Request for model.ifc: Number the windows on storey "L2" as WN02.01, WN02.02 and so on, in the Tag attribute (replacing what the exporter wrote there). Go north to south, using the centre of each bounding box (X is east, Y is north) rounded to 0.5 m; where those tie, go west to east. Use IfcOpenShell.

First a look at what the model holds.

```python
import ifcopenshell
import ifcopenshell.util.element
import ifcopenshell.util.placement

model = ifcopenshell.open("model.ifc")
print(model.schema)
storey = next(s for s in model.by_type("IfcBuildingStorey") if s.Name == "L2")
windows = [e for e in ifcopenshell.util.element.get_decomposition(storey) if e.is_a("IfcWindow")]
for e in sorted(windows, key=lambda e: e.id()):
    origin = ifcopenshell.util.placement.get_local_placement(e.ObjectPlacement)[:3, 3]
    print(e.id(), e.Tag, e.Name, origin.round(2) + 0.0, sep=" | ")
```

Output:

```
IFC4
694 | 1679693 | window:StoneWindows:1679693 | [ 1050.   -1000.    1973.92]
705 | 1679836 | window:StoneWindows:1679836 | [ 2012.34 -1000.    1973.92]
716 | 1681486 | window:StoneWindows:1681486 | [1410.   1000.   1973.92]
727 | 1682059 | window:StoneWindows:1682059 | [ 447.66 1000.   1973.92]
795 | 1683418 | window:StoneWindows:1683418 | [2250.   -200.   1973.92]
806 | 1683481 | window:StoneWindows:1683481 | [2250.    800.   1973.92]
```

```python
import ifcopenshell
import ifcopenshell.geom
import ifcopenshell.util.element
import ifcopenshell.util.shape

model = ifcopenshell.open("model.ifc")
settings = ifcopenshell.geom.settings()
settings.set("use-world-coords", True)


def centre(element):
    shape = ifcopenshell.geom.create_shape(settings, element)
    return ifcopenshell.util.shape.get_bbox_centroid(shape.geometry)


storey = next(s for s in model.by_type("IfcBuildingStorey") if s.Name == "L2")
windows = [e for e in ifcopenshell.util.element.get_decomposition(storey) if e.is_a("IfcWindow")]

# Insertion points can sit at a corner or the storey origin, so sort by the geometry (in metres).
centres = {e: centre(e) for e in windows}
windows.sort(key=lambda e: (-round(centres[e][1] / 0.5), centres[e][0]))

for i, e in enumerate(windows, start=1):
    number = f"WN02.{i:02d}"
    e.Tag = number
    print(e.id(), number)

model.write("model_updated.ifc")
```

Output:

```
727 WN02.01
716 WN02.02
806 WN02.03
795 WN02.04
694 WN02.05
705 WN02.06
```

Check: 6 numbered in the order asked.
